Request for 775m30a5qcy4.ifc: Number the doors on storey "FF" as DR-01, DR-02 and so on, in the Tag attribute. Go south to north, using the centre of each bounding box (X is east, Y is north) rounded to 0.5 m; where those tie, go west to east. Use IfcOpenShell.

First a look at what the model holds.

```python
import ifcopenshell
import ifcopenshell.util.element
import ifcopenshell.util.placement

model = ifcopenshell.open("775m30a5qcy4.ifc")
print(model.schema)
storey = next(s for s in model.by_type("IfcBuildingStorey") if s.Name == "FF")
doors = [e for e in ifcopenshell.util.element.get_decomposition(storey) if e.is_a("IfcDoor")]
for e in sorted(doors, key=lambda e: e.id()):
    origin = ifcopenshell.util.placement.get_local_placement(e.ObjectPlacement)[:3, 3]
    print(e.id(), e.Tag, e.Name, origin.round(2) + 0.0, sep=" | ")
```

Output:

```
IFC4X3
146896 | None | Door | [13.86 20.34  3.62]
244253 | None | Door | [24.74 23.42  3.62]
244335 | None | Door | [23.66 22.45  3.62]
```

```python
import ifcopenshell
import ifcopenshell.geom
import ifcopenshell.util.element
import ifcopenshell.util.shape

model = ifcopenshell.open("775m30a5qcy4.ifc")
settings = ifcopenshell.geom.settings()
settings.set("use-world-coords", True)


def centre(element):
    shape = ifcopenshell.geom.create_shape(settings, element)
    return ifcopenshell.util.shape.get_bbox_centroid(shape.geometry)


storey = next(s for s in model.by_type("IfcBuildingStorey") if s.Name == "FF")
doors = [e for e in ifcopenshell.util.element.get_decomposition(storey) if e.is_a("IfcDoor")]

# Insertion points can sit at a corner or the storey origin, so sort by the geometry (in metres).
centres = {e: centre(e) for e in doors}
doors.sort(key=lambda e: (round(centres[e][1] / 0.5), centres[e][0]))

for i, e in enumerate(doors, start=1):
    number = f"DR-{i:02d}"
    e.Tag = number
    print(e.id(), number)

model.write("775m30a5qcy4_updated.ifc")
```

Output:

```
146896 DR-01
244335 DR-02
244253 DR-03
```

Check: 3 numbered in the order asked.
